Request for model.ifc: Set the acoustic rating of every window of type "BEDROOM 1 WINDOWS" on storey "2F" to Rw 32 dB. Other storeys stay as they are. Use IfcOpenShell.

First a look at what the model holds.

```python
import ifcopenshell
import ifcopenshell.util.element

model = ifcopenshell.open("model.ifc")
print(model.schema)
storey = next(s for s in model.by_type("IfcBuildingStorey") if s.Name == "2F")
windows = [e for e in ifcopenshell.util.element.get_decomposition(storey) if e.is_a("IfcWindow")]
seen = {}
for e in windows:
    element_type = ifcopenshell.util.element.get_type(e)
    key = (element_type.Name if element_type != e and element_type else None, ifcopenshell.util.element.get_pset(e, "Pset_WindowCommon", "AcousticRating"))
    seen[key] = seen.get(key, 0) + 1
for (name, value), count in sorted(seen.items(), key=str):
    print(count, "x", name, "|", value)
```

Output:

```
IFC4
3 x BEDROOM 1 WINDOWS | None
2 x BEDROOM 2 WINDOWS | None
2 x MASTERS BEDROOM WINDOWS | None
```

```python
import ifcopenshell
import ifcopenshell.api.pset
import ifcopenshell.util.element

model = ifcopenshell.open("model.ifc")

storey = next(s for s in model.by_type("IfcBuildingStorey") if s.Name == "2F")
windows = [e for e in ifcopenshell.util.element.get_decomposition(storey) if e.is_a("IfcWindow")]

count = 0
for e in windows:
    element_type = ifcopenshell.util.element.get_type(e)
    if element_type in (None, e) or element_type.Name != "BEDROOM 1 WINDOWS":
        continue
    # add_pset returns the element's existing set when there is one.
    pset = ifcopenshell.api.pset.add_pset(model, product=e, name="Pset_WindowCommon")
    ifcopenshell.api.pset.edit_pset(model, pset=pset, properties={"AcousticRating": "Rw 32 dB"})
    count += 1

print(count, "windows updated")

model.write("model_updated.ifc")
```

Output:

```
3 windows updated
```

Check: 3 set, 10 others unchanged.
